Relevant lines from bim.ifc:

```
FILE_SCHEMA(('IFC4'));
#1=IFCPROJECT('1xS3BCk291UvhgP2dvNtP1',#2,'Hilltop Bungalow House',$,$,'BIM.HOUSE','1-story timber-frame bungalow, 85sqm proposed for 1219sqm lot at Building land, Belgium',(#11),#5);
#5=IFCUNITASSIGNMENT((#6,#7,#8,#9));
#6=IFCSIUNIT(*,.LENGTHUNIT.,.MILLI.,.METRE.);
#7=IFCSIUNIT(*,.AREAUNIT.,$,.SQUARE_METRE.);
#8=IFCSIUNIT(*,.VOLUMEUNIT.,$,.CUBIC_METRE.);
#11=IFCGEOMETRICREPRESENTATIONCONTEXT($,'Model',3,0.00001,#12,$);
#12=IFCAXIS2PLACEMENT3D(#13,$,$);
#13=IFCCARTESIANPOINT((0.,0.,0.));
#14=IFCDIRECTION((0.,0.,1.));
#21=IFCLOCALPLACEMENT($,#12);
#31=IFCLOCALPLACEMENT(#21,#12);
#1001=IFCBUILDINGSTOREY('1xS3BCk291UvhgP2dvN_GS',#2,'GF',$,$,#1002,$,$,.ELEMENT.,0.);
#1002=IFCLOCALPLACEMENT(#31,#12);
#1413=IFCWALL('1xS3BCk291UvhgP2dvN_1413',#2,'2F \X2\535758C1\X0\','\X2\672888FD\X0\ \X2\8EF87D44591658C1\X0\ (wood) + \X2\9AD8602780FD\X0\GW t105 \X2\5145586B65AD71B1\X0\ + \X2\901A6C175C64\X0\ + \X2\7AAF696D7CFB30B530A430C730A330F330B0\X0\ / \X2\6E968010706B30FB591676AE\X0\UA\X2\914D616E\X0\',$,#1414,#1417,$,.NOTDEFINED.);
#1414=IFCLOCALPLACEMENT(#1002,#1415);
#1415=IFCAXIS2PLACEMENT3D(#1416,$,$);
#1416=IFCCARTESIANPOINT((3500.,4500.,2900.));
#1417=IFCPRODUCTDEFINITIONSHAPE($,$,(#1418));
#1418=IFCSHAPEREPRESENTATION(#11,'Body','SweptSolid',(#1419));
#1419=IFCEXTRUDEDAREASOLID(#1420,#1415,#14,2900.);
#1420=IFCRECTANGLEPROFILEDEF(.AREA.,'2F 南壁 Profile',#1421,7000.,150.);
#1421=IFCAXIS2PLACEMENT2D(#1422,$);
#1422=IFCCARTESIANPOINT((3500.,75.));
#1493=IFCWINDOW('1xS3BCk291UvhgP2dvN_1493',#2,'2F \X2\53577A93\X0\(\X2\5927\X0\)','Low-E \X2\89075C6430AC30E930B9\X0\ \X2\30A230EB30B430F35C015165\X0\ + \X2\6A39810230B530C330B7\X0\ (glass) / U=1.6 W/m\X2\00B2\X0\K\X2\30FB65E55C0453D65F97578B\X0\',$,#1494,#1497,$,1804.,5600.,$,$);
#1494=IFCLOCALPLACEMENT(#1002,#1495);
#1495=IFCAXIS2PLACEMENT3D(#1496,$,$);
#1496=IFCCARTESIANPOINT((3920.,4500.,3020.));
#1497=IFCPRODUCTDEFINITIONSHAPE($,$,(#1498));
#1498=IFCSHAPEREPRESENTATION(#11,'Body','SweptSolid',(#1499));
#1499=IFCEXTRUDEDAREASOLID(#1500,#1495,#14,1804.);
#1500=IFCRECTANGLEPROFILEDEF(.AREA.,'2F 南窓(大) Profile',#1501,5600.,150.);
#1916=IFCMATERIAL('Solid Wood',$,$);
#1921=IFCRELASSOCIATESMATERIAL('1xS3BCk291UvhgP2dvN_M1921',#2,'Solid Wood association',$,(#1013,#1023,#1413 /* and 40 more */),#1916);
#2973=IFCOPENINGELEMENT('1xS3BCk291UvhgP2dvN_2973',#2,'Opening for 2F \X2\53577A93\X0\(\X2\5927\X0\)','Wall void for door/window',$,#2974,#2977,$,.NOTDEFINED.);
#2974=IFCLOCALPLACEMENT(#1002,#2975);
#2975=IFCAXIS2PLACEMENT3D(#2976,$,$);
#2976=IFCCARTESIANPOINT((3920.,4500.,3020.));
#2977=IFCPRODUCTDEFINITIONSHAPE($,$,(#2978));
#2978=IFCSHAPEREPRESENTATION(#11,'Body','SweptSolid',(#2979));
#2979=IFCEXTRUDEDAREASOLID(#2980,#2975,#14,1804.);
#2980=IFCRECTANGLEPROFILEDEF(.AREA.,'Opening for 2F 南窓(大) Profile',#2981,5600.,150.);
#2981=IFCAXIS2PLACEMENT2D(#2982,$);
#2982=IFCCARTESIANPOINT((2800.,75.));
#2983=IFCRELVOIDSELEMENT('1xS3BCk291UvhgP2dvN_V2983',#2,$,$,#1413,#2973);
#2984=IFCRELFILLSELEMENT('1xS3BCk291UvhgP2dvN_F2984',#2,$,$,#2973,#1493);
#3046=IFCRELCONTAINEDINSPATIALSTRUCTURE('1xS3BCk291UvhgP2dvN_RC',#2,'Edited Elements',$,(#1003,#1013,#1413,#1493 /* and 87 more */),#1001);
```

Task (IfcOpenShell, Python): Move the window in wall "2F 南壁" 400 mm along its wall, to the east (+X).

```python
import ifcopenshell
import ifcopenshell.api.geometry
import ifcopenshell.util.placement

model = ifcopenshell.open("bim.ifc")

window = model.by_guid("1xS3BCk291UvhgP2dvN_1493")
opening = window.FillsVoids[0].RelatingOpeningElement
wall = opening.VoidsElements[0].RelatingBuildingElement

wall_matrix = ifcopenshell.util.placement.get_local_placement(wall.ObjectPlacement)
shift = wall_matrix[:3, 0] * 400.0
before = ifcopenshell.util.placement.get_local_placement(window.ObjectPlacement)[:3, 3].copy()

# The window is not placed relative to its opening, so move both.
for product in (opening, window):
    matrix = ifcopenshell.util.placement.get_local_placement(product.ObjectPlacement)
    matrix[:3, 3] += shift
    ifcopenshell.api.geometry.edit_object_placement(model, product=product, matrix=matrix, is_si=False)

after = ifcopenshell.util.placement.get_local_placement(window.ObjectPlacement)[:3, 3]
print("window moved by", (after - before).round(3) + 0.0)

model.write("bim-out.ifc")
```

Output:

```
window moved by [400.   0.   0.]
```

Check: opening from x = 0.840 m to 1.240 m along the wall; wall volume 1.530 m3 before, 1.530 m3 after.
